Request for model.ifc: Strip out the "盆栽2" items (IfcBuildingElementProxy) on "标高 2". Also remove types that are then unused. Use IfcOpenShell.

First a look at what the model holds.

```python
import ifcopenshell
import ifcopenshell.util.element

model = ifcopenshell.open("model.ifc")
print(model.schema)
storey = next(s for s in model.by_type("IfcBuildingStorey") if s.Name == "标高 2")
proxies = [e for e in ifcopenshell.util.element.get_decomposition(storey) if e.is_a("IfcBuildingElementProxy")]
seen = {}
for e in proxies:
    element_type = ifcopenshell.util.element.get_type(e)
    name = element_type.Name if element_type not in (None, e) else None
    seen[name] = seen.get(name, 0) + 1
for name, count in sorted(seen.items(), key=str):
    print(count, "x", name)
```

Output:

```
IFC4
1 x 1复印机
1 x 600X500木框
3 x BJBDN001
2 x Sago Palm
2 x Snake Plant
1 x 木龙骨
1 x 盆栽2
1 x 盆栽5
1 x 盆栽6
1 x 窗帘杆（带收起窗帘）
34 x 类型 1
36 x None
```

```python
import ifcopenshell
import ifcopenshell.api.root
import ifcopenshell.util.element

model = ifcopenshell.open("model.ifc")

storey = next(s for s in model.by_type("IfcBuildingStorey") if s.Name == "标高 2")
proxies = [e for e in ifcopenshell.util.element.get_decomposition(storey) if e.is_a("IfcBuildingElementProxy")]
targets = [e for e in proxies if (t := ifcopenshell.util.element.get_type(e)) not in (None, e) and t.Name == "盆栽2"]
types = {ifcopenshell.util.element.get_type(e) for e in targets} - {None, *targets}

for e in targets:
    ifcopenshell.api.root.remove_product(model, product=e)
print(len(targets), "removed")

unused = [t for t in types if not ifcopenshell.util.element.get_types(t)]
for t in unused:
    ifcopenshell.api.root.remove_product(model, product=t)
print(len(unused), "unused types removed")

model.write("model_v2.ifc")
```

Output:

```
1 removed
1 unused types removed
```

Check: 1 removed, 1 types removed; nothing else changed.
